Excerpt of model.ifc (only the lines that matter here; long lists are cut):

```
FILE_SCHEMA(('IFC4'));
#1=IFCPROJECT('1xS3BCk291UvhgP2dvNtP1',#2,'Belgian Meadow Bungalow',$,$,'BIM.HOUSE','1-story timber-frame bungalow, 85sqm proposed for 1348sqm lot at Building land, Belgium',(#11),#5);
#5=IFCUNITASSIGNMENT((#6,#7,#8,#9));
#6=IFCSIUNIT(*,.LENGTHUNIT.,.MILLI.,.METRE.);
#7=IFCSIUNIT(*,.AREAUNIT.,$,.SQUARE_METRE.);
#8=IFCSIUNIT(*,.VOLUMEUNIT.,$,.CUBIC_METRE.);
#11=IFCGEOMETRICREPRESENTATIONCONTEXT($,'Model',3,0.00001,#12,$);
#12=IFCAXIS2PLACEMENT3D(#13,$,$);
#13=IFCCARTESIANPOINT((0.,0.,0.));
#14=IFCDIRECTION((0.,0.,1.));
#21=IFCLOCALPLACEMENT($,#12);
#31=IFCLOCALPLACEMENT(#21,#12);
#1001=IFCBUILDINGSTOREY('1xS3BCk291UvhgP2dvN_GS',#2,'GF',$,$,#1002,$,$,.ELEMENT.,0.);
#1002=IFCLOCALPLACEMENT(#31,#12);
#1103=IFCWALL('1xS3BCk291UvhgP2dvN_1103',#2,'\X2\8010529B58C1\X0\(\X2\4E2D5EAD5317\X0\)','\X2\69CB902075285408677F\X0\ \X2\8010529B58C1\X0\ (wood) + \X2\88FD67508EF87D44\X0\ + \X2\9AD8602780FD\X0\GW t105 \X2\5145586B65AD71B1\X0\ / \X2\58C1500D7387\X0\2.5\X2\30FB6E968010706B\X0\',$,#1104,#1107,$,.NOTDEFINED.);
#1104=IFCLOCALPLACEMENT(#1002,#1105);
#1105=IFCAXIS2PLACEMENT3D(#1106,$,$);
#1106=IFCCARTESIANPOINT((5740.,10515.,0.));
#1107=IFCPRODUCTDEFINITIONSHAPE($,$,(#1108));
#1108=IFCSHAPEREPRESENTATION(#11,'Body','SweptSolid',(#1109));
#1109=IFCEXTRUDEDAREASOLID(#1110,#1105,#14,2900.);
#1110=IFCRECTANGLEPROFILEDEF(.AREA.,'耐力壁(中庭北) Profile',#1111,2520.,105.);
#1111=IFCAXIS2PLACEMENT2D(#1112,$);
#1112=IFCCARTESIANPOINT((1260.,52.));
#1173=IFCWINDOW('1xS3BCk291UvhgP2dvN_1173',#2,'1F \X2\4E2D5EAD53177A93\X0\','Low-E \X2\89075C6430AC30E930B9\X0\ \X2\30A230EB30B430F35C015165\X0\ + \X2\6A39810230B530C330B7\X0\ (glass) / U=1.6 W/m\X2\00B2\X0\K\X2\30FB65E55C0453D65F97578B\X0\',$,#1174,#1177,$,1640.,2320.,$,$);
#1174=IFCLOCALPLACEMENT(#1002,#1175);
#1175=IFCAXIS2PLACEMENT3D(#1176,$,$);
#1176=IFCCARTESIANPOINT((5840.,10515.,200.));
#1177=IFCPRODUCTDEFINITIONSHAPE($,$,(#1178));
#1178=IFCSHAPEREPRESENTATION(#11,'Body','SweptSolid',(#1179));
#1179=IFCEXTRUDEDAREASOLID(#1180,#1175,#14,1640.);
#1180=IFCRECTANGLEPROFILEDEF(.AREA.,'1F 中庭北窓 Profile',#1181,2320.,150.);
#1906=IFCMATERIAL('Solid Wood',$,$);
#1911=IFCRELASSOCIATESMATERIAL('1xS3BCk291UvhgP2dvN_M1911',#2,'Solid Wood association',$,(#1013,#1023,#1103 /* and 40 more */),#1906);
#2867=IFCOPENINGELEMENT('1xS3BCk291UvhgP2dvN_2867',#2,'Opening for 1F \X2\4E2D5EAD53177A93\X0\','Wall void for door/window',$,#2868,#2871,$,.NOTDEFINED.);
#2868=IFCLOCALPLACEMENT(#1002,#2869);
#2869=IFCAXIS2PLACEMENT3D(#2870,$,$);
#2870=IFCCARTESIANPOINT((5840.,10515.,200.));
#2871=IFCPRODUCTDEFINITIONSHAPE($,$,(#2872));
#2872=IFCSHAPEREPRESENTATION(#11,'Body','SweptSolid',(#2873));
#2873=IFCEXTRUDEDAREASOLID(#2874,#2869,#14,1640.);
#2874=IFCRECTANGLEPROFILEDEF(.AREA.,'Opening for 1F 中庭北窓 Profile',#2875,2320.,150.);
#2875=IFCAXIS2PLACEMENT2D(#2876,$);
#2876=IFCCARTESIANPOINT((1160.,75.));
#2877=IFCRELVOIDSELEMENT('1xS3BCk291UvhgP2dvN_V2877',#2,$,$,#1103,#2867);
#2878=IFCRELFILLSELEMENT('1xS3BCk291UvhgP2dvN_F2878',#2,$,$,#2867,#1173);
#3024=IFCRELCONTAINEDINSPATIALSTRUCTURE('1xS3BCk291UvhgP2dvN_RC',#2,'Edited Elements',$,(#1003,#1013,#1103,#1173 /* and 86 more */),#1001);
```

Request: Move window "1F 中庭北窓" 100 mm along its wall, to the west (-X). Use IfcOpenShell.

```python
import ifcopenshell
import ifcopenshell.api.geometry
import ifcopenshell.util.placement
import ifcopenshell.util.unit

model = ifcopenshell.open("model.ifc")
unit_scale = ifcopenshell.util.unit.calculate_unit_scale(model)

window = model.by_guid("1xS3BCk291UvhgP2dvN_1173")
opening = window.FillsVoids[0].RelatingOpeningElement
wall = opening.VoidsElements[0].RelatingBuildingElement

wall_matrix = ifcopenshell.util.placement.get_local_placement(wall.ObjectPlacement)
shift = wall_matrix[:3, 0] * -0.1 / unit_scale
before = ifcopenshell.util.placement.get_local_placement(window.ObjectPlacement)[:3, 3].copy()

# The window is not placed relative to its opening, so move both.
for product in (opening, window):
    matrix = ifcopenshell.util.placement.get_local_placement(product.ObjectPlacement)
    matrix[:3, 3] += shift
    ifcopenshell.api.geometry.edit_object_placement(model, product=product, matrix=matrix, is_si=False)

after = ifcopenshell.util.placement.get_local_placement(window.ObjectPlacement)[:3, 3]
print("window moved by", (after - before).round(3) + 0.0)

model.write("model_v2.ifc")
```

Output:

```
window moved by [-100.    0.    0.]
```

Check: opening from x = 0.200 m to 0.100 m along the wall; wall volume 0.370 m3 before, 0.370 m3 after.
